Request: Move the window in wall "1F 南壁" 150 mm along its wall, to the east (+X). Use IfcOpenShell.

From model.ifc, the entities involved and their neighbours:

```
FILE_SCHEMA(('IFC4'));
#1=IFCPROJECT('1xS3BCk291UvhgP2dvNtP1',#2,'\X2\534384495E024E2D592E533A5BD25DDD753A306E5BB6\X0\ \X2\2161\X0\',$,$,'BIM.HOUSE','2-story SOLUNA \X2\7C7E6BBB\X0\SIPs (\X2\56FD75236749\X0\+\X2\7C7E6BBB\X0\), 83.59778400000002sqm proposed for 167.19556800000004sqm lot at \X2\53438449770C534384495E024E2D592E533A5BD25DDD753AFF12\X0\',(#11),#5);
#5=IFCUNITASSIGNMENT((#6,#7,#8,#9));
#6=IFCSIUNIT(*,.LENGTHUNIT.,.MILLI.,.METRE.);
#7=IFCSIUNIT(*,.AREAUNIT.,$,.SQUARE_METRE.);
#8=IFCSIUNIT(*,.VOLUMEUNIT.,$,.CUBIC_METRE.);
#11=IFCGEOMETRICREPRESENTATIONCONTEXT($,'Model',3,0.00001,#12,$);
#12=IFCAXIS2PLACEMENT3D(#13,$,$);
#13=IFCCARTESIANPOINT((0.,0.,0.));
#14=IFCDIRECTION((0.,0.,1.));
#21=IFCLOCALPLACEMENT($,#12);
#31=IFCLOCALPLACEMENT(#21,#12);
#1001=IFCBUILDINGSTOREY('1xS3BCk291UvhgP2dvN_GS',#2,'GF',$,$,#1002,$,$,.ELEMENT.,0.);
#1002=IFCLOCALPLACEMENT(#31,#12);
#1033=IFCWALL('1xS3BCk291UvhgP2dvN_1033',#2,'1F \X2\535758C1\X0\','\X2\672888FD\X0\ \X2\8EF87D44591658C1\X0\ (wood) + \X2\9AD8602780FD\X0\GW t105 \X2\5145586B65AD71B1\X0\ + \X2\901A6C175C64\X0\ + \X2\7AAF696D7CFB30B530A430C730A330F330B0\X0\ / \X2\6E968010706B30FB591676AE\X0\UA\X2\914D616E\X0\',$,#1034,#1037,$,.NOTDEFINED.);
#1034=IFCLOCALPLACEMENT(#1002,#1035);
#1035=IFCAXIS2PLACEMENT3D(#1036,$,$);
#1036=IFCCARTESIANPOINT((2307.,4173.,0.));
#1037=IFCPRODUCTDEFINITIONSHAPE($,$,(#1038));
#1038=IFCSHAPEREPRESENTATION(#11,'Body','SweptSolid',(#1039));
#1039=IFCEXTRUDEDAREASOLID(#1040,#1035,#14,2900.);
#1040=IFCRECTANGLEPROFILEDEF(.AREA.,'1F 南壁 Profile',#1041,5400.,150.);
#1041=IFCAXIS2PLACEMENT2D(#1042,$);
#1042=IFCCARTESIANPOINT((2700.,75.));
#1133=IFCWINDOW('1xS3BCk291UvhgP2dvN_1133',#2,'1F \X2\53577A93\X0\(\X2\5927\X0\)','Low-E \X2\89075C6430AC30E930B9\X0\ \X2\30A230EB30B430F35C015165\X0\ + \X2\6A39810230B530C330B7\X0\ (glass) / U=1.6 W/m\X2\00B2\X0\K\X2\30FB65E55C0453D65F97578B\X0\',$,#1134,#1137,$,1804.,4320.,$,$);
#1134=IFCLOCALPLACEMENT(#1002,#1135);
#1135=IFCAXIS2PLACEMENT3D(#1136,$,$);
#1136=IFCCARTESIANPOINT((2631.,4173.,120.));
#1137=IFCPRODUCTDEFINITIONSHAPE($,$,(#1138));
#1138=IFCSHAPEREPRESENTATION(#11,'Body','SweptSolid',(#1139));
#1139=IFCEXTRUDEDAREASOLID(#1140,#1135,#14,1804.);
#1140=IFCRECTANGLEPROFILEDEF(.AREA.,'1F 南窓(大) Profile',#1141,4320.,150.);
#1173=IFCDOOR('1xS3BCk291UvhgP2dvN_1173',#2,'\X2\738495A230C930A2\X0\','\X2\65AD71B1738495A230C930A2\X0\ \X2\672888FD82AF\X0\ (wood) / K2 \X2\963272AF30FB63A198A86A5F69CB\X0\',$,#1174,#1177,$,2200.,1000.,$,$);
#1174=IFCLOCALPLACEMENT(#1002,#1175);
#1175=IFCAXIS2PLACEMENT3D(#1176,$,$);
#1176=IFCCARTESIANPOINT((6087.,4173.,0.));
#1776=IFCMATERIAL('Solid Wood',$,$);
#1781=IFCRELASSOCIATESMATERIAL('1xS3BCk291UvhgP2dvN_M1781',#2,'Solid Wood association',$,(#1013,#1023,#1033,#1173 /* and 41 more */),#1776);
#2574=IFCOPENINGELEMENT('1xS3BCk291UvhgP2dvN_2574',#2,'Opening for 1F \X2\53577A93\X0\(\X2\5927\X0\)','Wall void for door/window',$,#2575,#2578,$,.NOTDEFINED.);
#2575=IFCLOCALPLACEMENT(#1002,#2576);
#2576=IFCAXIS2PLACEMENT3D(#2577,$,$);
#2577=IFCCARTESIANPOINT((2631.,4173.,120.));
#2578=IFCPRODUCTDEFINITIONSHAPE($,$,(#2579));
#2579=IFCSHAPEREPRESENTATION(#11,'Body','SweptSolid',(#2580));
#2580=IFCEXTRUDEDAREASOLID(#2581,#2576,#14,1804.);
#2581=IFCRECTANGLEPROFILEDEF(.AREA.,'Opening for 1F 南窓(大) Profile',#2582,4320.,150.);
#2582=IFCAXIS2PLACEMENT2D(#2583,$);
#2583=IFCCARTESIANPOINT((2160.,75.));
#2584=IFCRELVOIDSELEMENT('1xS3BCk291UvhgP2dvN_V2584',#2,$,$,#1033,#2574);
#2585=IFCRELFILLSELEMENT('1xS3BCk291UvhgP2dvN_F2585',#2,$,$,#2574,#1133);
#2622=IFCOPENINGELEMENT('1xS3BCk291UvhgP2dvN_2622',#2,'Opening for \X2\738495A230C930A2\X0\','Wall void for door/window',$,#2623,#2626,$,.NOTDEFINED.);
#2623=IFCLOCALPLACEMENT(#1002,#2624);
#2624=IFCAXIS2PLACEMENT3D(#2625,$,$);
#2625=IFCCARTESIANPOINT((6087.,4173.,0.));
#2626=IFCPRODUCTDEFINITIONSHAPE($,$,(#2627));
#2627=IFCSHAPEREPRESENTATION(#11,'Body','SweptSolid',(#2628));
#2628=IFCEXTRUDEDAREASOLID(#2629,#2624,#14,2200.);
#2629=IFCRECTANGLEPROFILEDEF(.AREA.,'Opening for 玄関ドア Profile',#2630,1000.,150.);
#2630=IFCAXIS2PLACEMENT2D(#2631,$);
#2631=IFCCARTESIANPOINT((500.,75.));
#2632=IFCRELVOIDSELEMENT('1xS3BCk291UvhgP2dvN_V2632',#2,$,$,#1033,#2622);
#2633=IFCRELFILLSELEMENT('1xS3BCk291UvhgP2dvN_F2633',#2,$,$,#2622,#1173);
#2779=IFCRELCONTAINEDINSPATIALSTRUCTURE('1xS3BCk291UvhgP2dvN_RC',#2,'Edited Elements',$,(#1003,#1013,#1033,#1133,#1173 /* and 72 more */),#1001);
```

```python
import ifcopenshell
import ifcopenshell.api.geometry
import ifcopenshell.util.placement
import ifcopenshell.util.unit

model = ifcopenshell.open("model.ifc")
unit_scale = ifcopenshell.util.unit.calculate_unit_scale(model)

window = model.by_id(1133)
opening = window.FillsVoids[0].RelatingOpeningElement
wall = opening.VoidsElements[0].RelatingBuildingElement

wall_matrix = ifcopenshell.util.placement.get_local_placement(wall.ObjectPlacement)
shift = wall_matrix[:3, 0] * 0.15 / unit_scale
before = ifcopenshell.util.placement.get_local_placement(window.ObjectPlacement)[:3, 3].copy()

# The window is not placed relative to its opening, so move both.
for product in (opening, window):
    matrix = ifcopenshell.util.placement.get_local_placement(product.ObjectPlacement)
    matrix[:3, 3] += shift
    ifcopenshell.api.geometry.edit_object_placement(model, product=product, matrix=matrix, is_si=False)

after = ifcopenshell.util.placement.get_local_placement(window.ObjectPlacement)[:3, 3]
print("window moved by", (after - before).round(3) + 0.0)

model.write("model-out.ifc")
```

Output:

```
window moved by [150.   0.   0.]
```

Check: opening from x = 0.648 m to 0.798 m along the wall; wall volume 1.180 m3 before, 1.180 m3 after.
